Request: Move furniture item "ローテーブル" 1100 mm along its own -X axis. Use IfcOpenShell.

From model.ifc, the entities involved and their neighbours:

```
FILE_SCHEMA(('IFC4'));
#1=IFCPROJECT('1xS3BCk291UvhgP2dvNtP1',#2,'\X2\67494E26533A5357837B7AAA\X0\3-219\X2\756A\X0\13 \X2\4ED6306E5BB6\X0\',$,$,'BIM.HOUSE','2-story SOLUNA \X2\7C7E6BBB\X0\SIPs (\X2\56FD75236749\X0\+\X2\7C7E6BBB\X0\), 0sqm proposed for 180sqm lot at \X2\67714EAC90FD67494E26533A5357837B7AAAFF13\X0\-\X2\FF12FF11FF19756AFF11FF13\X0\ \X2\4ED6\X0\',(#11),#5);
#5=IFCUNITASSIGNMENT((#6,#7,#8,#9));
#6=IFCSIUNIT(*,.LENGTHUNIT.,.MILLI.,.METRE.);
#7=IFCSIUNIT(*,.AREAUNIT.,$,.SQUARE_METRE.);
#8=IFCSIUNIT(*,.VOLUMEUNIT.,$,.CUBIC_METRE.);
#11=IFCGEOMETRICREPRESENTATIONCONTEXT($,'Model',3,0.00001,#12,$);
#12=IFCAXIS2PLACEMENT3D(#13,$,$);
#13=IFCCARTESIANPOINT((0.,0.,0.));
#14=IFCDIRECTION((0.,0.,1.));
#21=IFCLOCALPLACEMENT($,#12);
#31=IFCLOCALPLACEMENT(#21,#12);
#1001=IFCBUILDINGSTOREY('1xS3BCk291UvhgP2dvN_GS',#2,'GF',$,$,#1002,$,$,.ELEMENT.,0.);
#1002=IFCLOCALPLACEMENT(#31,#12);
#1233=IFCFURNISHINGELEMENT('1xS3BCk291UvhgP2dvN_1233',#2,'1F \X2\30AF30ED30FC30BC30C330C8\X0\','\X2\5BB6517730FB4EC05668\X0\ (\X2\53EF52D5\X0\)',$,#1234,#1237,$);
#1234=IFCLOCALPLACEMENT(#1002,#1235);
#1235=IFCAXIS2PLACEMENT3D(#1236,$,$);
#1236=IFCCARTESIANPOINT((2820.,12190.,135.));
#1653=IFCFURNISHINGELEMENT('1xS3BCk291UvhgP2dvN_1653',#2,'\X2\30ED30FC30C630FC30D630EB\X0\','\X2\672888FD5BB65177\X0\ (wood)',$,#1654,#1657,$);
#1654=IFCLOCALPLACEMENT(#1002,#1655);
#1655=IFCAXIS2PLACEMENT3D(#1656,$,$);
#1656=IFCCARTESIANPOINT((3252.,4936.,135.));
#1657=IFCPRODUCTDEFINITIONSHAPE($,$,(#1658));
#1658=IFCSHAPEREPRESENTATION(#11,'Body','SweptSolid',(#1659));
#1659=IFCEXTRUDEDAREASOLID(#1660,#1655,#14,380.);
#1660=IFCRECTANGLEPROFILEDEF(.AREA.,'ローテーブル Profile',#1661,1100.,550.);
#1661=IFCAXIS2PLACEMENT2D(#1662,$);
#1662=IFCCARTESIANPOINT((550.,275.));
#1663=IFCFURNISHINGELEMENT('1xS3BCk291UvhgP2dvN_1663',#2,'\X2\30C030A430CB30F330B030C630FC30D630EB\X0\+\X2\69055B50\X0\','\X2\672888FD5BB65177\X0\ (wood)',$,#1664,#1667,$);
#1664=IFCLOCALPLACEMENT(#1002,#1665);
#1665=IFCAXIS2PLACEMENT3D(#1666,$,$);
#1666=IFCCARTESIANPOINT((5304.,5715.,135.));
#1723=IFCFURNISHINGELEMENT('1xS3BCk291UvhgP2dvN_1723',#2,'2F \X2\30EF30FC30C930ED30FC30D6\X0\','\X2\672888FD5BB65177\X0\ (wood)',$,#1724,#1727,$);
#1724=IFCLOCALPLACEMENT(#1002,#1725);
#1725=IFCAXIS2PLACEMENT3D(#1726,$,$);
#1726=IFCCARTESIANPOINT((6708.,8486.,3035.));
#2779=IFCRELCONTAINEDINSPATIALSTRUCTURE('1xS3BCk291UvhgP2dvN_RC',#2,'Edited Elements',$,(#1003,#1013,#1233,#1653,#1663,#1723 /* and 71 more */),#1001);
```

```python
import ifcopenshell
import ifcopenshell.api.geometry
import ifcopenshell.util.placement
import ifcopenshell.util.unit

model = ifcopenshell.open("model.ifc")
unit_scale = ifcopenshell.util.unit.calculate_unit_scale(model)

item = model.by_guid("1xS3BCk291UvhgP2dvN_1653")
matrix = ifcopenshell.util.placement.get_local_placement(item.ObjectPlacement)
matrix[:3, 3] -= matrix[:3, 0] * 1.1 / unit_scale
ifcopenshell.api.geometry.edit_object_placement(model, product=item, matrix=matrix, is_si=False)

print(ifcopenshell.util.placement.get_local_placement(item.ObjectPlacement).round(3) + 0.0)

model.write("model_v2.ifc")
```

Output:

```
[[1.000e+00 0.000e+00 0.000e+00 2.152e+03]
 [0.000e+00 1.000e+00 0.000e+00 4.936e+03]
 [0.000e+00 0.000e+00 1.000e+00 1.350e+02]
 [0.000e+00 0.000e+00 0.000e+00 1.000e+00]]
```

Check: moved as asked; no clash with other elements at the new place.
